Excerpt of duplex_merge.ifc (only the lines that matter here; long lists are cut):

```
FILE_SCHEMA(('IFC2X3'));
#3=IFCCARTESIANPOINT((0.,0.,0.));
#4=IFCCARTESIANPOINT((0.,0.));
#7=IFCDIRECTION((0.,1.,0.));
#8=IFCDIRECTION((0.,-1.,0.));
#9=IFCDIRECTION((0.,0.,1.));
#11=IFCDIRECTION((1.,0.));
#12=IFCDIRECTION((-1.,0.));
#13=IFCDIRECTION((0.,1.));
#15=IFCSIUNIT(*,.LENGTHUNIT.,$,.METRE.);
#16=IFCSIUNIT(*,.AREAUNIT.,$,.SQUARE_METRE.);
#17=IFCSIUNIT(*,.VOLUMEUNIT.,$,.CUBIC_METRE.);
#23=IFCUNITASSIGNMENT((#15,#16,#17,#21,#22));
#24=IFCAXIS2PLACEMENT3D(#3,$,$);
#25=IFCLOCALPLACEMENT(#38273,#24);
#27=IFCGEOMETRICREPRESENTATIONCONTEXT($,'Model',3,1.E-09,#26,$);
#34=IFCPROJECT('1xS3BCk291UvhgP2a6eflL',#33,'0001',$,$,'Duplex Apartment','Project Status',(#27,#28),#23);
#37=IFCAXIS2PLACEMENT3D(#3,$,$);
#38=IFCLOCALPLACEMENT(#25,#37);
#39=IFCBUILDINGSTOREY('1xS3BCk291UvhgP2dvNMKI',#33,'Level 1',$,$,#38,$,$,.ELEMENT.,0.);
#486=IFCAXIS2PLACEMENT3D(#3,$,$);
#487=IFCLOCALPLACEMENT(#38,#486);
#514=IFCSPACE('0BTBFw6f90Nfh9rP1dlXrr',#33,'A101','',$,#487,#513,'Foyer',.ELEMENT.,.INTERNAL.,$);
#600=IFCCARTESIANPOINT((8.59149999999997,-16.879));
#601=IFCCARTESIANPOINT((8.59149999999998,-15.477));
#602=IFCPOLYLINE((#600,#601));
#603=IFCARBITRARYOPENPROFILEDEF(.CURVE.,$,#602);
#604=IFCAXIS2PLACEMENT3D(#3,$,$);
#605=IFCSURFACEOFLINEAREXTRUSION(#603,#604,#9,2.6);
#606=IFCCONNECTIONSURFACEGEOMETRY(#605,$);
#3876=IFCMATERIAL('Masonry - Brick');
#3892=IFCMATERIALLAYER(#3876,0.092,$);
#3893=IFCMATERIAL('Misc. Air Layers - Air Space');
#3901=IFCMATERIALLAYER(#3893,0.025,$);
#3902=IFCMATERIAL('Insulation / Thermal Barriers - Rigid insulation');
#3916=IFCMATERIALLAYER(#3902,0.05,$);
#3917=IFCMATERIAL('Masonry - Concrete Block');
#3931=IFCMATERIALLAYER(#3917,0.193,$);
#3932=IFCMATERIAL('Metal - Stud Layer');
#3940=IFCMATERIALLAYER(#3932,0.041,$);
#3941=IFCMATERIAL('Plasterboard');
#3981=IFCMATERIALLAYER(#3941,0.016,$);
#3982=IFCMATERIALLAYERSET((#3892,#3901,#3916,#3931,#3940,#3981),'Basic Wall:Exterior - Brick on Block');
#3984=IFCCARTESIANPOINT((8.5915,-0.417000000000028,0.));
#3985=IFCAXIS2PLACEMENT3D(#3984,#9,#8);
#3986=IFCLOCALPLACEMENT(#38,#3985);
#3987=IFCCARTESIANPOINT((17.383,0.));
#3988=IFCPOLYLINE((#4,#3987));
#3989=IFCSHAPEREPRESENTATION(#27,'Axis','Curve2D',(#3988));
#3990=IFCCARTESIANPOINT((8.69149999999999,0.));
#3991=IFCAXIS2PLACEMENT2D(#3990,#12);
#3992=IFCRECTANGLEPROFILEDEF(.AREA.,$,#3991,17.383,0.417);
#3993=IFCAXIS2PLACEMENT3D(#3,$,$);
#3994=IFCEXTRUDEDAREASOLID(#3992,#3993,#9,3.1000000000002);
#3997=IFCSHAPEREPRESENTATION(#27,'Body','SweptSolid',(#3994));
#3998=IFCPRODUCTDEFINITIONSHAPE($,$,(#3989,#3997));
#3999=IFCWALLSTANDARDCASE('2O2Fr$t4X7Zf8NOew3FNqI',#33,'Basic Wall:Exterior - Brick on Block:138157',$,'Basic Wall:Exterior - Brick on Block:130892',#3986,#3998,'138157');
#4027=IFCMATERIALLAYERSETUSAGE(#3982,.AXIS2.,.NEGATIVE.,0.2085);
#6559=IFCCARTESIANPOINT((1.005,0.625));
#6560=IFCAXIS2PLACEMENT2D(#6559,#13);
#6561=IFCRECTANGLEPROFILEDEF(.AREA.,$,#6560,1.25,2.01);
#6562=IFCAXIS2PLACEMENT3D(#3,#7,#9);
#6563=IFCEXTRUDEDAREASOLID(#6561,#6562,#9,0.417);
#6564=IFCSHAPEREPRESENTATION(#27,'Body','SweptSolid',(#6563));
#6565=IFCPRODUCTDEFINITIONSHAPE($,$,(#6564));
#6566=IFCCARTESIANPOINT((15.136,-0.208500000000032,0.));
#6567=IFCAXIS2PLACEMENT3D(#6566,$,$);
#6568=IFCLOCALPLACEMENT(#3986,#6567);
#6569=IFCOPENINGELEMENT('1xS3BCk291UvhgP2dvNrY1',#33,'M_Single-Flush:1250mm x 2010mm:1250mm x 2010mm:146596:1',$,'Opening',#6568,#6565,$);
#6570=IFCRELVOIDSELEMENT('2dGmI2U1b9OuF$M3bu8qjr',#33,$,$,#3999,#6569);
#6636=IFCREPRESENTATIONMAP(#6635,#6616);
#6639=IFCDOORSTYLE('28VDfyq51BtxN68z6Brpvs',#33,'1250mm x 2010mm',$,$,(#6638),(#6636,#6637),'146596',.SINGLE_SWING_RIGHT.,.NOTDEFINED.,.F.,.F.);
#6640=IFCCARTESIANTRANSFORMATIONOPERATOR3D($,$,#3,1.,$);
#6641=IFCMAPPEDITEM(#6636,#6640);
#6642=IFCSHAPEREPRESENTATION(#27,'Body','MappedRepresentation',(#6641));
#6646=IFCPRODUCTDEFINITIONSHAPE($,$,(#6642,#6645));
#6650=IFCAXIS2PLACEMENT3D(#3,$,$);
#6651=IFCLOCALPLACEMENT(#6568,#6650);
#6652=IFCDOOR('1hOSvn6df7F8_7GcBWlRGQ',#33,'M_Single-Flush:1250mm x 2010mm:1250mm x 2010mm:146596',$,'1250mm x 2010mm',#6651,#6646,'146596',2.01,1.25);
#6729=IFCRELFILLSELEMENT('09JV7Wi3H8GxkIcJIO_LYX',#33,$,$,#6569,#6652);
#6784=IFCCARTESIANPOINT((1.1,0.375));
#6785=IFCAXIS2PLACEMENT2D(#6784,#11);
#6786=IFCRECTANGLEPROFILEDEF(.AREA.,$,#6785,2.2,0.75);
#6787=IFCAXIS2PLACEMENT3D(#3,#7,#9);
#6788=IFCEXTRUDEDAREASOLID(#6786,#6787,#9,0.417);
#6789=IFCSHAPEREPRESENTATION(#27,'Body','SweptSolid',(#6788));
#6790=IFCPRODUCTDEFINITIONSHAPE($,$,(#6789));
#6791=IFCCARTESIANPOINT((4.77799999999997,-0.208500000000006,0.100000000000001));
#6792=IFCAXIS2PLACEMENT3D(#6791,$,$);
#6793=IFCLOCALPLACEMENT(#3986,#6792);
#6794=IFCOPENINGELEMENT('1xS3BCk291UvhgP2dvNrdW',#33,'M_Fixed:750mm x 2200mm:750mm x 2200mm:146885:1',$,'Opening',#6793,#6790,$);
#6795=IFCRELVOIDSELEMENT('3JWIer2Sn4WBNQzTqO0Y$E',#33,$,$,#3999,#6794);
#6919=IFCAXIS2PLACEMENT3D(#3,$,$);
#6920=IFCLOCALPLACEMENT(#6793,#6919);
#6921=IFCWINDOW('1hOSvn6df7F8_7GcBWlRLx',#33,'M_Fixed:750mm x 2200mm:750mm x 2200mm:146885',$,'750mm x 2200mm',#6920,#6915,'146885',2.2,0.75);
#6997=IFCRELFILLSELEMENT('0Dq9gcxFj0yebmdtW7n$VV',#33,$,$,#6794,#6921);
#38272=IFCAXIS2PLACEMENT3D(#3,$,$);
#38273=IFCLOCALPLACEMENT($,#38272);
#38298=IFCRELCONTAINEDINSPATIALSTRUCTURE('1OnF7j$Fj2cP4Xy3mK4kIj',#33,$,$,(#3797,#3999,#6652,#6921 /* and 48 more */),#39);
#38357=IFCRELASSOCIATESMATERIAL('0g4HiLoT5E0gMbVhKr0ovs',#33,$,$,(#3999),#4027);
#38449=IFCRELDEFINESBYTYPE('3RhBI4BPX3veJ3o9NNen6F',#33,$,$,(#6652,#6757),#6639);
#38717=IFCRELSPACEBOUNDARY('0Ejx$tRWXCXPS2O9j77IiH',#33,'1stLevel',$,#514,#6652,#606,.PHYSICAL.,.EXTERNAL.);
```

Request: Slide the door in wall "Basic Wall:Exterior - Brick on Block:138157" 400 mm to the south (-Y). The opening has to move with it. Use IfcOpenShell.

```python
import numpy as np
import ifcopenshell
import ifcopenshell.api.geometry
import ifcopenshell.util.placement

model = ifcopenshell.open("duplex_merge.ifc")

door = model.by_id(6652)
opening = door.FillsVoids[0].RelatingOpeningElement
wall = opening.VoidsElements[0].RelatingBuildingElement

wall_matrix = ifcopenshell.util.placement.get_local_placement(wall.ObjectPlacement)
shift = wall_matrix[:3, 0] * 0.4
before = ifcopenshell.util.placement.get_local_placement(door.ObjectPlacement)[:3, 3].copy()

# The door is placed relative to its opening, so it follows when the opening moves.
matrix = ifcopenshell.util.placement.get_local_placement(opening.ObjectPlacement)
matrix[:3, 3] += shift
ifcopenshell.api.geometry.edit_object_placement(
    model, product=opening, matrix=matrix, is_si=False, should_transform_children=True
)

# Space boundary surfaces are stored in each space's coordinates; move them too.
for rel in door.ProvidesBoundaries:
    if not rel.ConnectionGeometry:
        continue
    surface = rel.ConnectionGeometry.SurfaceOnRelatingElement
    space_matrix = ifcopenshell.util.placement.get_local_placement(rel.RelatingSpace.ObjectPlacement)
    point = np.array(surface.Position.Location.Coordinates) + space_matrix[:3, :3].T @ shift
    surface.Position = model.createIfcAxis2Placement3D(
        model.createIfcCartesianPoint(point.tolist()), surface.Position.Axis, surface.Position.RefDirection
    )

after = ifcopenshell.util.placement.get_local_placement(door.ObjectPlacement)[:3, 3]
print("door moved by", (after - before).round(3) + 0.0)

model.write("duplex_merge_v2.ifc")
```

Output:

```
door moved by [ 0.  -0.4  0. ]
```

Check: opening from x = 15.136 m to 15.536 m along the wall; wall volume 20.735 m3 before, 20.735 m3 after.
